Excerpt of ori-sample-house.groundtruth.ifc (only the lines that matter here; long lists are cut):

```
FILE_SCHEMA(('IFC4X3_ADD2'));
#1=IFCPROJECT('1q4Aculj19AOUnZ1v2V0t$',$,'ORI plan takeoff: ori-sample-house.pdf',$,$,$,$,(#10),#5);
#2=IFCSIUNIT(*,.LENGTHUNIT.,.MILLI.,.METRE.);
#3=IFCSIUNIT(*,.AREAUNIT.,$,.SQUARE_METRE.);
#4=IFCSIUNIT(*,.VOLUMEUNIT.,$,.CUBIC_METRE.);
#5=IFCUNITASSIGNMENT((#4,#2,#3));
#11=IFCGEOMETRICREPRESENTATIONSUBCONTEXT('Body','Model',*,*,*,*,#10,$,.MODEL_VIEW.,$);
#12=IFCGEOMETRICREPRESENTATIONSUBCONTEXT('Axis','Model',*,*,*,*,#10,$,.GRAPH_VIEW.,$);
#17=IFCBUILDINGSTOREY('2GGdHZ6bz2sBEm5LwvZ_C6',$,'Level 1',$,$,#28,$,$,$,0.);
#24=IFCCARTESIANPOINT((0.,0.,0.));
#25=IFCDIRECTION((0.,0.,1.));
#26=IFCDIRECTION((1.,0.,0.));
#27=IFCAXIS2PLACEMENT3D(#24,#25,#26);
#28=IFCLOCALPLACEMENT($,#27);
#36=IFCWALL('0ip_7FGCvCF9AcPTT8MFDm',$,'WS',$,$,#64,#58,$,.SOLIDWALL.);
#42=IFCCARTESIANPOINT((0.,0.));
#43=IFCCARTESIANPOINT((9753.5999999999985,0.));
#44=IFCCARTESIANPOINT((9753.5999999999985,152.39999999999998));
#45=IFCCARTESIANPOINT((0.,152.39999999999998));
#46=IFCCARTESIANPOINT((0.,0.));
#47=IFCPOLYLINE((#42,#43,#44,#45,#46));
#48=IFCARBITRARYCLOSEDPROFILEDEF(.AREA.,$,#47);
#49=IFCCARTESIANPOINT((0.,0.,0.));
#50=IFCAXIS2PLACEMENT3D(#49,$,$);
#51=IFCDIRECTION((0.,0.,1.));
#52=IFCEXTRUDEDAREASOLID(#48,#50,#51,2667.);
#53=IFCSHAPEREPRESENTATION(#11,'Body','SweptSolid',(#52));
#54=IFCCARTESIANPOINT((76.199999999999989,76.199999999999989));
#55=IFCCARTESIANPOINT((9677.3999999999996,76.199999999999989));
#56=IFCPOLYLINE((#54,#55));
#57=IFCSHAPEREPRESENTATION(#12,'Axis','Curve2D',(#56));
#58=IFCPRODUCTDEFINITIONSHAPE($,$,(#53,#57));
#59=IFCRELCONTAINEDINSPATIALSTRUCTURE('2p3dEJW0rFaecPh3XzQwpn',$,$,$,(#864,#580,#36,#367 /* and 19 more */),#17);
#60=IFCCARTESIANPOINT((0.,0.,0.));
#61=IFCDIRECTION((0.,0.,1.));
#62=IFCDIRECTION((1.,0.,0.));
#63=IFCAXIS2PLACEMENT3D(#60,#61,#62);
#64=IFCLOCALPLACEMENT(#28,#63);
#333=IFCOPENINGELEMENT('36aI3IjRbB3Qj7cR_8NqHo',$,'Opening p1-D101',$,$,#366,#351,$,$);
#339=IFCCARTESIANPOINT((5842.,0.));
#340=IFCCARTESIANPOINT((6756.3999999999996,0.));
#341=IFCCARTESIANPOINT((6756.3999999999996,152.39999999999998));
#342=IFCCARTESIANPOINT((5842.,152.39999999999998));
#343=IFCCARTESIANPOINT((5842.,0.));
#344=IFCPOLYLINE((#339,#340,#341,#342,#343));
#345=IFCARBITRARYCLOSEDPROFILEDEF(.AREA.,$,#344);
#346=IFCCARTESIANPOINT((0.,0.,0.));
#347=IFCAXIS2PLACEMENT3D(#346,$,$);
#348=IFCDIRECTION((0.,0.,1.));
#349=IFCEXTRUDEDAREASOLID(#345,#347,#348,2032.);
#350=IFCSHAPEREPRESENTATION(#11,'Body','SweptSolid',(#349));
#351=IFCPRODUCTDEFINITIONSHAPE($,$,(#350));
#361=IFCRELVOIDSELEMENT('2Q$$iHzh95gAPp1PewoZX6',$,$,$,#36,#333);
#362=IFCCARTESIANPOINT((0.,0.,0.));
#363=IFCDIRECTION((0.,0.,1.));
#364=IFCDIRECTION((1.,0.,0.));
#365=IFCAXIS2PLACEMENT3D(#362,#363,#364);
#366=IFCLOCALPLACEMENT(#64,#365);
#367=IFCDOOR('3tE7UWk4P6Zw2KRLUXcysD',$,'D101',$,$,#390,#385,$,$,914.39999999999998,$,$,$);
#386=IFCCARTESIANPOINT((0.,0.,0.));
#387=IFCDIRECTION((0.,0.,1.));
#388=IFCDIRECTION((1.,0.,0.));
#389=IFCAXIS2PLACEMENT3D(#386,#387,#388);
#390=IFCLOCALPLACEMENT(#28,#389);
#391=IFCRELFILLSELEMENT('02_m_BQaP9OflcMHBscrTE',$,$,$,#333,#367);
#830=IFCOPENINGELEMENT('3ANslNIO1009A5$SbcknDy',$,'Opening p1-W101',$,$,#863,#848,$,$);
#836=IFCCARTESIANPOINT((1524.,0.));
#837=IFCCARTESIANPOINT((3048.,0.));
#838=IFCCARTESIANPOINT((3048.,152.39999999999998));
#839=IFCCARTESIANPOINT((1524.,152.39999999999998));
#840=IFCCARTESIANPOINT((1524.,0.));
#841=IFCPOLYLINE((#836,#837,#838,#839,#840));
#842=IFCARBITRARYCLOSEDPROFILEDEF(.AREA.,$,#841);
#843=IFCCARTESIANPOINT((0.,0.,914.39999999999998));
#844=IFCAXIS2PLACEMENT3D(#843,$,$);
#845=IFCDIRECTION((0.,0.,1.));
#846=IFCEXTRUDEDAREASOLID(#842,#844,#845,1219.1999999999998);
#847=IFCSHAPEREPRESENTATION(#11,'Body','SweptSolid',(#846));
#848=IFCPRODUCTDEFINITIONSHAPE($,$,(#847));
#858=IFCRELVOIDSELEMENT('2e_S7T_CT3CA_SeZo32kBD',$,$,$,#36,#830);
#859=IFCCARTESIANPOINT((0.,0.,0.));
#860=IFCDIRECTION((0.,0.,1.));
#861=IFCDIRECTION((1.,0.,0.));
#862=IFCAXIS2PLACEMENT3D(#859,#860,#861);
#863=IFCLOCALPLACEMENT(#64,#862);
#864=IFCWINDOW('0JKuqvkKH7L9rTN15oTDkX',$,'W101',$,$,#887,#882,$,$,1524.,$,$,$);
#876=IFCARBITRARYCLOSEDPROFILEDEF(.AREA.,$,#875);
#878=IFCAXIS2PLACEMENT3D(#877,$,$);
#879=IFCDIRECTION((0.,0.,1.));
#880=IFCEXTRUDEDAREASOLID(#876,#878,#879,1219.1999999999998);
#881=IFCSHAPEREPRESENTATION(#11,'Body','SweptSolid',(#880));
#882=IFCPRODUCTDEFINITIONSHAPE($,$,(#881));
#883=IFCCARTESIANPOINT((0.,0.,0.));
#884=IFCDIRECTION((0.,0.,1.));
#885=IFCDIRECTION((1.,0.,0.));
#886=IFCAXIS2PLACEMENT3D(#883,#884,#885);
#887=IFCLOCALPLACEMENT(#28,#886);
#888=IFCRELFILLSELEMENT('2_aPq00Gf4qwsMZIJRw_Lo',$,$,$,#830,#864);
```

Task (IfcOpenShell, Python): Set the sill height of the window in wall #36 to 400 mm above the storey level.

```python
import numpy as np
import ifcopenshell
import ifcopenshell.api.geometry
import ifcopenshell.geom
import ifcopenshell.util.element
import ifcopenshell.util.placement
import ifcopenshell.util.shape
import ifcopenshell.util.unit

model = ifcopenshell.open("ori-sample-house.groundtruth.ifc")
unit_scale = ifcopenshell.util.unit.calculate_unit_scale(model)

window = model.by_id(864)
opening = window.FillsVoids[0].RelatingOpeningElement
storey = ifcopenshell.util.element.get_container(window, ifc_class="IfcBuildingStorey")
level = ifcopenshell.util.placement.get_local_placement(storey.ObjectPlacement)[2, 3]

# The opening's origin need not be at the sill, so measure its lowest point.
shape = ifcopenshell.geom.create_shape(ifcopenshell.geom.settings(), opening)
bottom = ifcopenshell.util.shape.get_shape_bottom_elevation(shape, shape.geometry) / unit_scale
dz = level + 400.0 - bottom

shift = np.array([0.0, 0.0, dz])
# The window is not placed relative to its opening, so move both.
for product in (opening, window):
    matrix = ifcopenshell.util.placement.get_local_placement(product.ObjectPlacement)
    matrix[:3, 3] += shift
    ifcopenshell.api.geometry.edit_object_placement(model, product=product, matrix=matrix, is_si=False)

print(f"moved by {dz * unit_scale:+.3f} m")

model.write("ori-sample-house.groundtruth_edited.ifc")
```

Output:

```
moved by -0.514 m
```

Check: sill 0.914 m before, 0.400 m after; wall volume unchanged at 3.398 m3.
